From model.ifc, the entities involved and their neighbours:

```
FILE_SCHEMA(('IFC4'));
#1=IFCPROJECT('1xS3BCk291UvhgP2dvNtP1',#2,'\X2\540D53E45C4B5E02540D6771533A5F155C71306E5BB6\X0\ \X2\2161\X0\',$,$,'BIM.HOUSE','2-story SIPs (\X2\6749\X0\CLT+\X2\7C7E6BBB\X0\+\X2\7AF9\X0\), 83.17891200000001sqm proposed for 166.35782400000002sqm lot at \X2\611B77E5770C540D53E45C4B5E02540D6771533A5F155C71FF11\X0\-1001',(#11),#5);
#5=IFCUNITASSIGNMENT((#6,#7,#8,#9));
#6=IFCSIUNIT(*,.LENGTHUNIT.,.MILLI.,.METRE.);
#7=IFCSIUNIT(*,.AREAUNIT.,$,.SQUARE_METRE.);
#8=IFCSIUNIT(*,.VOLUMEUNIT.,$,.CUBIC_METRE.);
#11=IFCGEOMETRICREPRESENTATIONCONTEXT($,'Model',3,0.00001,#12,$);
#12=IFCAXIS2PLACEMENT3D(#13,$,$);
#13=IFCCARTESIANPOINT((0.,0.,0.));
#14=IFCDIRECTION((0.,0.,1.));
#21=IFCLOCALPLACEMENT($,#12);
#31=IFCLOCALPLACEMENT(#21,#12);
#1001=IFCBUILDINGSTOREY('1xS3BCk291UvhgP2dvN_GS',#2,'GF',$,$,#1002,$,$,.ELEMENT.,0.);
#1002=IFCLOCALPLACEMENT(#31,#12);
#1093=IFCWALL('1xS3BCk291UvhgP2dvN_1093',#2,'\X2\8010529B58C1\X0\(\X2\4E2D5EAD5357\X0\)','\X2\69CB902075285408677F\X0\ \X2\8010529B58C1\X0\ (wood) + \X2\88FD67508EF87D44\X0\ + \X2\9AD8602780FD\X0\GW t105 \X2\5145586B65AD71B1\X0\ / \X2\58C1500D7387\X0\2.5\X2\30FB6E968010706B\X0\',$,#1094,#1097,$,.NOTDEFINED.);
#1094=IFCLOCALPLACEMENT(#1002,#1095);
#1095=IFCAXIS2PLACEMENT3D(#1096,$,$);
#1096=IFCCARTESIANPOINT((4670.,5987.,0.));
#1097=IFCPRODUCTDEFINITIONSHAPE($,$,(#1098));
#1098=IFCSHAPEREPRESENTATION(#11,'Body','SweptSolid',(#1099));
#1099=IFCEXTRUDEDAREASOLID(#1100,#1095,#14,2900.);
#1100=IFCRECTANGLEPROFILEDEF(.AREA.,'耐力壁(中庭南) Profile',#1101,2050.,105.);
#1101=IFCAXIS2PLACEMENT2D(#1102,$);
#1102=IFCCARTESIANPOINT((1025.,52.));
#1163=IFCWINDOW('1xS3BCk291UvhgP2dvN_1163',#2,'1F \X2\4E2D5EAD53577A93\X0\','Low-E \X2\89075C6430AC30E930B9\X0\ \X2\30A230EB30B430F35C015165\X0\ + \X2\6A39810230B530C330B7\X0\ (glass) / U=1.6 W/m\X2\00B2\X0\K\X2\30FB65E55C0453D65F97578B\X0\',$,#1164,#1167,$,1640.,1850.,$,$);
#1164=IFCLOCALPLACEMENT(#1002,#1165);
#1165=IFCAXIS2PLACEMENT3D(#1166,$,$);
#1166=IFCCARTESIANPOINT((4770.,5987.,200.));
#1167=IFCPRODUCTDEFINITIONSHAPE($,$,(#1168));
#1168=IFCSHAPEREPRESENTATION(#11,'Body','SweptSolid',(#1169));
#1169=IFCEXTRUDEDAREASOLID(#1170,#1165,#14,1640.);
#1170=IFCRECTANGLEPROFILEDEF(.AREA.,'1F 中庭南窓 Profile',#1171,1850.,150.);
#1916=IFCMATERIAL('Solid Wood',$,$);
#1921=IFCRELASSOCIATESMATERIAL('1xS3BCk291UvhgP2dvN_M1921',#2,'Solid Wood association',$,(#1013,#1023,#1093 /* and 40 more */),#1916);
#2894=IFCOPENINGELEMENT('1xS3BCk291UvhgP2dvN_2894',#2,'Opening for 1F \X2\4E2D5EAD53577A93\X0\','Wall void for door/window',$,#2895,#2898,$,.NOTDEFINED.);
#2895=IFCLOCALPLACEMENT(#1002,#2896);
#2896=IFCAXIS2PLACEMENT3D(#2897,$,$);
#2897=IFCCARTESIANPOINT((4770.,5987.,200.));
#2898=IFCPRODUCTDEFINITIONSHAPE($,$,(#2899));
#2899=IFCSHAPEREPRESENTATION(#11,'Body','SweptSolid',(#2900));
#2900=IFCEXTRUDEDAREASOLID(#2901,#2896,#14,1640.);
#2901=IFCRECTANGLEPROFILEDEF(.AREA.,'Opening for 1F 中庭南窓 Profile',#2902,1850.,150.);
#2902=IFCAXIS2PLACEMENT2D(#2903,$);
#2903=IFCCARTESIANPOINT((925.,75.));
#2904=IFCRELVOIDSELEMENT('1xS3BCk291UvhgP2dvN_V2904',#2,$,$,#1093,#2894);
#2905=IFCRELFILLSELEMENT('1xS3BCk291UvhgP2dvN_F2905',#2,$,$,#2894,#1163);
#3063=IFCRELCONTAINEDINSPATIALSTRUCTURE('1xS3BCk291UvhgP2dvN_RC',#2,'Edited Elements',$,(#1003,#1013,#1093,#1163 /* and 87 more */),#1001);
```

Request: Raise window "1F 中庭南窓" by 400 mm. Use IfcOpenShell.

```python
import numpy as np
import ifcopenshell
import ifcopenshell.api.geometry
import ifcopenshell.util.placement
import ifcopenshell.util.unit

model = ifcopenshell.open("model.ifc")
unit_scale = ifcopenshell.util.unit.calculate_unit_scale(model)

window = model.by_guid("1xS3BCk291UvhgP2dvN_1163")
opening = window.FillsVoids[0].RelatingOpeningElement
dz = 0.4 / unit_scale

shift = np.array([0.0, 0.0, dz])
# The window is not placed relative to its opening, so move both.
for product in (opening, window):
    matrix = ifcopenshell.util.placement.get_local_placement(product.ObjectPlacement)
    matrix[:3, 3] += shift
    ifcopenshell.api.geometry.edit_object_placement(model, product=product, matrix=matrix, is_si=False)

print(f"moved by {dz * unit_scale:+.3f} m")

model.write("model_edited.ifc")
```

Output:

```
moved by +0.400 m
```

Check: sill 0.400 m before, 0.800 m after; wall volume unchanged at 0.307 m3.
